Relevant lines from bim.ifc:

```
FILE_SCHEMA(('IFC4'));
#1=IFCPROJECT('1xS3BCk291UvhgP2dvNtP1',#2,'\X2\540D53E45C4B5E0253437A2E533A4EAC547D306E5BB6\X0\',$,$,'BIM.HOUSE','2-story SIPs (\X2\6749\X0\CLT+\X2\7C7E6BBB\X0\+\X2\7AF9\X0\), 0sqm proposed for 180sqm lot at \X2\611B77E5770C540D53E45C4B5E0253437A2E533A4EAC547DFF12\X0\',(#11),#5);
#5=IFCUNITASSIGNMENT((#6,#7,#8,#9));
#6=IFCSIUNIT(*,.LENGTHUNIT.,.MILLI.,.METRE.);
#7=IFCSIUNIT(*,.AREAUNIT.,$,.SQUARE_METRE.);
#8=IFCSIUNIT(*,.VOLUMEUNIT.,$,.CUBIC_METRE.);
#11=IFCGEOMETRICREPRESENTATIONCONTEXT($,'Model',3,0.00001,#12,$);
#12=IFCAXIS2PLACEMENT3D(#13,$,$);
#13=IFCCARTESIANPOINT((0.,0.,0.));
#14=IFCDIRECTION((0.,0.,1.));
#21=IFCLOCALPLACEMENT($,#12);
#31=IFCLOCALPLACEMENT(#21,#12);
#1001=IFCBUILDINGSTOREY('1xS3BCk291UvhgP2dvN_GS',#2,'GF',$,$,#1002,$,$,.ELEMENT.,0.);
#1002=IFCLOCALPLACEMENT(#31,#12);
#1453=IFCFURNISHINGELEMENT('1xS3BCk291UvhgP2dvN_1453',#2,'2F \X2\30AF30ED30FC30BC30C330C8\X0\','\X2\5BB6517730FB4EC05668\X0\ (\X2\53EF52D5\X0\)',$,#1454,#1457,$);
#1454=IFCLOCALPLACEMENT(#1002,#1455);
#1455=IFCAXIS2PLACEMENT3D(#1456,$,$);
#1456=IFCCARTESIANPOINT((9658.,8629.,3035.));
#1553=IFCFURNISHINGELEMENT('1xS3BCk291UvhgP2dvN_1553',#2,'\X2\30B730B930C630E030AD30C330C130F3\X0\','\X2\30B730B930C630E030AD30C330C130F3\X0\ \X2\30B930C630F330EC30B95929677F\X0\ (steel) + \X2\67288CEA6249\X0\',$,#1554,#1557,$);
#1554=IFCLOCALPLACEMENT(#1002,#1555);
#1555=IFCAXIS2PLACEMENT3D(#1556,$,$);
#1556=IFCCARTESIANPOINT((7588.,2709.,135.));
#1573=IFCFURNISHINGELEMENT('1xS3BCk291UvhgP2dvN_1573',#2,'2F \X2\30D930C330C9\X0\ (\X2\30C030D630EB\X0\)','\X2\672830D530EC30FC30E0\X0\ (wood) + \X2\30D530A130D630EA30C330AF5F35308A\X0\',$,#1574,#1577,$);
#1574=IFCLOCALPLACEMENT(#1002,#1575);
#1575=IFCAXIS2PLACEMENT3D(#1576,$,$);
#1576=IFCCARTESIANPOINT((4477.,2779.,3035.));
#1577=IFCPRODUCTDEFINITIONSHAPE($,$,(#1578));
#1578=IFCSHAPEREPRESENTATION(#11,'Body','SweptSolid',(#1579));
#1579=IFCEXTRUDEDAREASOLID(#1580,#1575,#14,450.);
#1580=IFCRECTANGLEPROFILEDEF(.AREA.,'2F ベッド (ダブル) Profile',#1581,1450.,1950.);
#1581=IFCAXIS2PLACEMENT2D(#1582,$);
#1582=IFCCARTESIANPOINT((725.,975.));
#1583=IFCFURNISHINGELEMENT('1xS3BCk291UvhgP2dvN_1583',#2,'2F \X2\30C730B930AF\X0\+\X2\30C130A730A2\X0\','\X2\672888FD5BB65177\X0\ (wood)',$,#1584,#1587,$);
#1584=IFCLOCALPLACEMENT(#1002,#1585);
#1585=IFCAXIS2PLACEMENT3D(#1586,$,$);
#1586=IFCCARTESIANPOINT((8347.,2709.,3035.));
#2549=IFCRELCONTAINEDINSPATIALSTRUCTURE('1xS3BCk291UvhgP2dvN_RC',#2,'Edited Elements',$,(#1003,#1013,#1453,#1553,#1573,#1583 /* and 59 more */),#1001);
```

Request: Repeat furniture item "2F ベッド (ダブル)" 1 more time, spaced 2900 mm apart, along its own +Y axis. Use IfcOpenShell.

```python
import ifcopenshell
import ifcopenshell.api.geometry
import ifcopenshell.api.root
import ifcopenshell.util.element
import ifcopenshell.util.placement
import ifcopenshell.util.unit

model = ifcopenshell.open("bim.ifc")
unit_scale = ifcopenshell.util.unit.calculate_unit_scale(model)


def reuse_history(source, copy):
    """copy_class also copies each property set's owner history, people and application; keep the originals."""
    for rel in copy.IsDefinedBy:
        if rel.is_a("IfcRelDefinesByProperties") and (history := rel.RelatingPropertyDefinition.OwnerHistory):
            rel.RelatingPropertyDefinition.OwnerHistory = source.OwnerHistory
            ifcopenshell.util.element.remove_deep2(model, history)


source = model.by_guid("1xS3BCk291UvhgP2dvN_1573")
base = ifcopenshell.util.placement.get_local_placement(source.ObjectPlacement)
step = base[:3, 1] * 2.9 / unit_scale

for i in range(1, 2):
    copy = ifcopenshell.api.root.copy_class(model, product=source)
    copy.Representation = ifcopenshell.util.element.copy_deep(
        model, source.Representation, exclude=["IfcGeometricRepresentationContext", "IfcRepresentationMap"]
    )
    reuse_history(source, copy)
    matrix = base.copy()
    matrix[:3, 3] += i * step
    print("added at", matrix[:3, 3].round(3) + 0.0)
    ifcopenshell.api.geometry.edit_object_placement(model, product=copy, matrix=matrix, is_si=False)

model.write("bim_v2.ifc")
```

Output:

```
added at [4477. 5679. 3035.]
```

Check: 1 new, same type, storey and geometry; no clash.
